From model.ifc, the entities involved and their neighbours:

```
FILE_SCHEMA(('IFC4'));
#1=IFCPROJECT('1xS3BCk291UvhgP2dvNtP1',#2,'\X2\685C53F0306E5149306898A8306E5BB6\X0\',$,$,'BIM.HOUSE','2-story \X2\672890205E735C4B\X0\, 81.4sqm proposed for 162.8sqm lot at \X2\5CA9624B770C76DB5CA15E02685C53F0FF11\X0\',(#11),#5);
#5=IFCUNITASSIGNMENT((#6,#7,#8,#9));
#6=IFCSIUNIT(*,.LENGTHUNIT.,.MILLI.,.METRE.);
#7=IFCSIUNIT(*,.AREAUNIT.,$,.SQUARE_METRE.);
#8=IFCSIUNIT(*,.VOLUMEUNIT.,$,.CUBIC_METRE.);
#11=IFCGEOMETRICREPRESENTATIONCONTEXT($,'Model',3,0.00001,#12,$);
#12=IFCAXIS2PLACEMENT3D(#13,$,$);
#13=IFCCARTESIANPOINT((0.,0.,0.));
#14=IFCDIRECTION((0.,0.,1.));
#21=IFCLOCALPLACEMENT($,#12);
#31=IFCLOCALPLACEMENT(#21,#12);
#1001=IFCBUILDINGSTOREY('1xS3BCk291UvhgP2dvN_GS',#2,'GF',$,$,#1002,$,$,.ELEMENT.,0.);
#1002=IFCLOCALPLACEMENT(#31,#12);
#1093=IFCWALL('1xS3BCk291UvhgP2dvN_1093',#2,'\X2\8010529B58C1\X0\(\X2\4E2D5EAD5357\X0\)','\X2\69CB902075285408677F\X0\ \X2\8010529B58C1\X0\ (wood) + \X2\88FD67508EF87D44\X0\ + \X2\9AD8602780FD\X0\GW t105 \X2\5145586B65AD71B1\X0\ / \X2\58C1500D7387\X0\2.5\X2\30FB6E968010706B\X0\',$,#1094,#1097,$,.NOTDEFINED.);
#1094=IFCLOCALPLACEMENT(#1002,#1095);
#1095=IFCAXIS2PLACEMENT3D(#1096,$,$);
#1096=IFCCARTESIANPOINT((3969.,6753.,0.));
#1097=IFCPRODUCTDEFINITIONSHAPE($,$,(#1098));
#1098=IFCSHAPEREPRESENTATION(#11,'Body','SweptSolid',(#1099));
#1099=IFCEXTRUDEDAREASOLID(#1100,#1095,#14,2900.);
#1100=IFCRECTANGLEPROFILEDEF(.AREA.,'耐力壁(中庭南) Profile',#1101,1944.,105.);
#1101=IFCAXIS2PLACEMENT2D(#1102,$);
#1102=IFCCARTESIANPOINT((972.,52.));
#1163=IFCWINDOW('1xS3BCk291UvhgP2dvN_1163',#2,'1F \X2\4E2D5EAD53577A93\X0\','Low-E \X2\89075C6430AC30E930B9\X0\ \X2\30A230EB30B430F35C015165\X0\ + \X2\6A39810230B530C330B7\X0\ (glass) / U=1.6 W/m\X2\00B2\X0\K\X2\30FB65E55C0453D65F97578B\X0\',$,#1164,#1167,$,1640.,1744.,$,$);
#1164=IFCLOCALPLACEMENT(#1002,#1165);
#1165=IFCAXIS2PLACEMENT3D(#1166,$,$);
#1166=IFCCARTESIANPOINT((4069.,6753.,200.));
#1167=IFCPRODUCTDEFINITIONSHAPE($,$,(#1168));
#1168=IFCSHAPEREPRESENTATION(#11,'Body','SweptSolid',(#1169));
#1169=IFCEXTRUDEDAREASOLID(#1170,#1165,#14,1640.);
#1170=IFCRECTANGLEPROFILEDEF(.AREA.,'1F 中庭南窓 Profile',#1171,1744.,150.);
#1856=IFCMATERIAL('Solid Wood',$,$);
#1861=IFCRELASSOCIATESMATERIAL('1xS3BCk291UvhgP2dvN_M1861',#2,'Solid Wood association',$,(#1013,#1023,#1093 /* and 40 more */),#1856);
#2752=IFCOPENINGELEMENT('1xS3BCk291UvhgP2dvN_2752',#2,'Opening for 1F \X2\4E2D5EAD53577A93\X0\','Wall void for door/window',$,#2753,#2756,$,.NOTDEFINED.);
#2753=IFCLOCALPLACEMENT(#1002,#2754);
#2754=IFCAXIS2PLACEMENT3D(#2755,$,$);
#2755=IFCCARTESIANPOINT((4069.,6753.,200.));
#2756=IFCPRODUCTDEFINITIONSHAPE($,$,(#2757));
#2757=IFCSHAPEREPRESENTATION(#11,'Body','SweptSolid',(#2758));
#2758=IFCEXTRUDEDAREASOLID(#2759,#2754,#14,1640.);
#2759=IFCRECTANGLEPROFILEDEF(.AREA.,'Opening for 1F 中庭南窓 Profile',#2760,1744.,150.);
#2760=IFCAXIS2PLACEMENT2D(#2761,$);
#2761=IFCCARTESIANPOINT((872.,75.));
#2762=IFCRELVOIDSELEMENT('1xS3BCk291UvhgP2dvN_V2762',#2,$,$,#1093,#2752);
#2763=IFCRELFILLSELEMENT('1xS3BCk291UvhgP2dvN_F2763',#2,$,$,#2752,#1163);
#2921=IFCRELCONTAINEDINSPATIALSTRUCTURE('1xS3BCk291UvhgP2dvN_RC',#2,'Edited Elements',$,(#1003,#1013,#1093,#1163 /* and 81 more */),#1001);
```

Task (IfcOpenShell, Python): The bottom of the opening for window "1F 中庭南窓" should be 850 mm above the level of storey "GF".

```python
import numpy as np
import ifcopenshell
import ifcopenshell.api.geometry
import ifcopenshell.geom
import ifcopenshell.util.element
import ifcopenshell.util.placement
import ifcopenshell.util.shape
import ifcopenshell.util.unit

model = ifcopenshell.open("model.ifc")
unit_scale = ifcopenshell.util.unit.calculate_unit_scale(model)

window = model.by_id(1163)
opening = window.FillsVoids[0].RelatingOpeningElement
storey = ifcopenshell.util.element.get_container(window, ifc_class="IfcBuildingStorey")
level = ifcopenshell.util.placement.get_local_placement(storey.ObjectPlacement)[2, 3]

# The opening's origin need not be at the sill, so measure its lowest point.
shape = ifcopenshell.geom.create_shape(ifcopenshell.geom.settings(), opening)
bottom = ifcopenshell.util.shape.get_shape_bottom_elevation(shape, shape.geometry) / unit_scale
dz = level + 0.85 / unit_scale - bottom

shift = np.array([0.0, 0.0, dz])
# The window is not placed relative to its opening, so move both.
for product in (opening, window):
    matrix = ifcopenshell.util.placement.get_local_placement(product.ObjectPlacement)
    matrix[:3, 3] += shift
    ifcopenshell.api.geometry.edit_object_placement(model, product=product, matrix=matrix, is_si=False)

print(f"moved by {dz * unit_scale:+.3f} m")

model.write("model_edited.ifc")
```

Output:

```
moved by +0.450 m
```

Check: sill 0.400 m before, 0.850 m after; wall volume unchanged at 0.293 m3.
